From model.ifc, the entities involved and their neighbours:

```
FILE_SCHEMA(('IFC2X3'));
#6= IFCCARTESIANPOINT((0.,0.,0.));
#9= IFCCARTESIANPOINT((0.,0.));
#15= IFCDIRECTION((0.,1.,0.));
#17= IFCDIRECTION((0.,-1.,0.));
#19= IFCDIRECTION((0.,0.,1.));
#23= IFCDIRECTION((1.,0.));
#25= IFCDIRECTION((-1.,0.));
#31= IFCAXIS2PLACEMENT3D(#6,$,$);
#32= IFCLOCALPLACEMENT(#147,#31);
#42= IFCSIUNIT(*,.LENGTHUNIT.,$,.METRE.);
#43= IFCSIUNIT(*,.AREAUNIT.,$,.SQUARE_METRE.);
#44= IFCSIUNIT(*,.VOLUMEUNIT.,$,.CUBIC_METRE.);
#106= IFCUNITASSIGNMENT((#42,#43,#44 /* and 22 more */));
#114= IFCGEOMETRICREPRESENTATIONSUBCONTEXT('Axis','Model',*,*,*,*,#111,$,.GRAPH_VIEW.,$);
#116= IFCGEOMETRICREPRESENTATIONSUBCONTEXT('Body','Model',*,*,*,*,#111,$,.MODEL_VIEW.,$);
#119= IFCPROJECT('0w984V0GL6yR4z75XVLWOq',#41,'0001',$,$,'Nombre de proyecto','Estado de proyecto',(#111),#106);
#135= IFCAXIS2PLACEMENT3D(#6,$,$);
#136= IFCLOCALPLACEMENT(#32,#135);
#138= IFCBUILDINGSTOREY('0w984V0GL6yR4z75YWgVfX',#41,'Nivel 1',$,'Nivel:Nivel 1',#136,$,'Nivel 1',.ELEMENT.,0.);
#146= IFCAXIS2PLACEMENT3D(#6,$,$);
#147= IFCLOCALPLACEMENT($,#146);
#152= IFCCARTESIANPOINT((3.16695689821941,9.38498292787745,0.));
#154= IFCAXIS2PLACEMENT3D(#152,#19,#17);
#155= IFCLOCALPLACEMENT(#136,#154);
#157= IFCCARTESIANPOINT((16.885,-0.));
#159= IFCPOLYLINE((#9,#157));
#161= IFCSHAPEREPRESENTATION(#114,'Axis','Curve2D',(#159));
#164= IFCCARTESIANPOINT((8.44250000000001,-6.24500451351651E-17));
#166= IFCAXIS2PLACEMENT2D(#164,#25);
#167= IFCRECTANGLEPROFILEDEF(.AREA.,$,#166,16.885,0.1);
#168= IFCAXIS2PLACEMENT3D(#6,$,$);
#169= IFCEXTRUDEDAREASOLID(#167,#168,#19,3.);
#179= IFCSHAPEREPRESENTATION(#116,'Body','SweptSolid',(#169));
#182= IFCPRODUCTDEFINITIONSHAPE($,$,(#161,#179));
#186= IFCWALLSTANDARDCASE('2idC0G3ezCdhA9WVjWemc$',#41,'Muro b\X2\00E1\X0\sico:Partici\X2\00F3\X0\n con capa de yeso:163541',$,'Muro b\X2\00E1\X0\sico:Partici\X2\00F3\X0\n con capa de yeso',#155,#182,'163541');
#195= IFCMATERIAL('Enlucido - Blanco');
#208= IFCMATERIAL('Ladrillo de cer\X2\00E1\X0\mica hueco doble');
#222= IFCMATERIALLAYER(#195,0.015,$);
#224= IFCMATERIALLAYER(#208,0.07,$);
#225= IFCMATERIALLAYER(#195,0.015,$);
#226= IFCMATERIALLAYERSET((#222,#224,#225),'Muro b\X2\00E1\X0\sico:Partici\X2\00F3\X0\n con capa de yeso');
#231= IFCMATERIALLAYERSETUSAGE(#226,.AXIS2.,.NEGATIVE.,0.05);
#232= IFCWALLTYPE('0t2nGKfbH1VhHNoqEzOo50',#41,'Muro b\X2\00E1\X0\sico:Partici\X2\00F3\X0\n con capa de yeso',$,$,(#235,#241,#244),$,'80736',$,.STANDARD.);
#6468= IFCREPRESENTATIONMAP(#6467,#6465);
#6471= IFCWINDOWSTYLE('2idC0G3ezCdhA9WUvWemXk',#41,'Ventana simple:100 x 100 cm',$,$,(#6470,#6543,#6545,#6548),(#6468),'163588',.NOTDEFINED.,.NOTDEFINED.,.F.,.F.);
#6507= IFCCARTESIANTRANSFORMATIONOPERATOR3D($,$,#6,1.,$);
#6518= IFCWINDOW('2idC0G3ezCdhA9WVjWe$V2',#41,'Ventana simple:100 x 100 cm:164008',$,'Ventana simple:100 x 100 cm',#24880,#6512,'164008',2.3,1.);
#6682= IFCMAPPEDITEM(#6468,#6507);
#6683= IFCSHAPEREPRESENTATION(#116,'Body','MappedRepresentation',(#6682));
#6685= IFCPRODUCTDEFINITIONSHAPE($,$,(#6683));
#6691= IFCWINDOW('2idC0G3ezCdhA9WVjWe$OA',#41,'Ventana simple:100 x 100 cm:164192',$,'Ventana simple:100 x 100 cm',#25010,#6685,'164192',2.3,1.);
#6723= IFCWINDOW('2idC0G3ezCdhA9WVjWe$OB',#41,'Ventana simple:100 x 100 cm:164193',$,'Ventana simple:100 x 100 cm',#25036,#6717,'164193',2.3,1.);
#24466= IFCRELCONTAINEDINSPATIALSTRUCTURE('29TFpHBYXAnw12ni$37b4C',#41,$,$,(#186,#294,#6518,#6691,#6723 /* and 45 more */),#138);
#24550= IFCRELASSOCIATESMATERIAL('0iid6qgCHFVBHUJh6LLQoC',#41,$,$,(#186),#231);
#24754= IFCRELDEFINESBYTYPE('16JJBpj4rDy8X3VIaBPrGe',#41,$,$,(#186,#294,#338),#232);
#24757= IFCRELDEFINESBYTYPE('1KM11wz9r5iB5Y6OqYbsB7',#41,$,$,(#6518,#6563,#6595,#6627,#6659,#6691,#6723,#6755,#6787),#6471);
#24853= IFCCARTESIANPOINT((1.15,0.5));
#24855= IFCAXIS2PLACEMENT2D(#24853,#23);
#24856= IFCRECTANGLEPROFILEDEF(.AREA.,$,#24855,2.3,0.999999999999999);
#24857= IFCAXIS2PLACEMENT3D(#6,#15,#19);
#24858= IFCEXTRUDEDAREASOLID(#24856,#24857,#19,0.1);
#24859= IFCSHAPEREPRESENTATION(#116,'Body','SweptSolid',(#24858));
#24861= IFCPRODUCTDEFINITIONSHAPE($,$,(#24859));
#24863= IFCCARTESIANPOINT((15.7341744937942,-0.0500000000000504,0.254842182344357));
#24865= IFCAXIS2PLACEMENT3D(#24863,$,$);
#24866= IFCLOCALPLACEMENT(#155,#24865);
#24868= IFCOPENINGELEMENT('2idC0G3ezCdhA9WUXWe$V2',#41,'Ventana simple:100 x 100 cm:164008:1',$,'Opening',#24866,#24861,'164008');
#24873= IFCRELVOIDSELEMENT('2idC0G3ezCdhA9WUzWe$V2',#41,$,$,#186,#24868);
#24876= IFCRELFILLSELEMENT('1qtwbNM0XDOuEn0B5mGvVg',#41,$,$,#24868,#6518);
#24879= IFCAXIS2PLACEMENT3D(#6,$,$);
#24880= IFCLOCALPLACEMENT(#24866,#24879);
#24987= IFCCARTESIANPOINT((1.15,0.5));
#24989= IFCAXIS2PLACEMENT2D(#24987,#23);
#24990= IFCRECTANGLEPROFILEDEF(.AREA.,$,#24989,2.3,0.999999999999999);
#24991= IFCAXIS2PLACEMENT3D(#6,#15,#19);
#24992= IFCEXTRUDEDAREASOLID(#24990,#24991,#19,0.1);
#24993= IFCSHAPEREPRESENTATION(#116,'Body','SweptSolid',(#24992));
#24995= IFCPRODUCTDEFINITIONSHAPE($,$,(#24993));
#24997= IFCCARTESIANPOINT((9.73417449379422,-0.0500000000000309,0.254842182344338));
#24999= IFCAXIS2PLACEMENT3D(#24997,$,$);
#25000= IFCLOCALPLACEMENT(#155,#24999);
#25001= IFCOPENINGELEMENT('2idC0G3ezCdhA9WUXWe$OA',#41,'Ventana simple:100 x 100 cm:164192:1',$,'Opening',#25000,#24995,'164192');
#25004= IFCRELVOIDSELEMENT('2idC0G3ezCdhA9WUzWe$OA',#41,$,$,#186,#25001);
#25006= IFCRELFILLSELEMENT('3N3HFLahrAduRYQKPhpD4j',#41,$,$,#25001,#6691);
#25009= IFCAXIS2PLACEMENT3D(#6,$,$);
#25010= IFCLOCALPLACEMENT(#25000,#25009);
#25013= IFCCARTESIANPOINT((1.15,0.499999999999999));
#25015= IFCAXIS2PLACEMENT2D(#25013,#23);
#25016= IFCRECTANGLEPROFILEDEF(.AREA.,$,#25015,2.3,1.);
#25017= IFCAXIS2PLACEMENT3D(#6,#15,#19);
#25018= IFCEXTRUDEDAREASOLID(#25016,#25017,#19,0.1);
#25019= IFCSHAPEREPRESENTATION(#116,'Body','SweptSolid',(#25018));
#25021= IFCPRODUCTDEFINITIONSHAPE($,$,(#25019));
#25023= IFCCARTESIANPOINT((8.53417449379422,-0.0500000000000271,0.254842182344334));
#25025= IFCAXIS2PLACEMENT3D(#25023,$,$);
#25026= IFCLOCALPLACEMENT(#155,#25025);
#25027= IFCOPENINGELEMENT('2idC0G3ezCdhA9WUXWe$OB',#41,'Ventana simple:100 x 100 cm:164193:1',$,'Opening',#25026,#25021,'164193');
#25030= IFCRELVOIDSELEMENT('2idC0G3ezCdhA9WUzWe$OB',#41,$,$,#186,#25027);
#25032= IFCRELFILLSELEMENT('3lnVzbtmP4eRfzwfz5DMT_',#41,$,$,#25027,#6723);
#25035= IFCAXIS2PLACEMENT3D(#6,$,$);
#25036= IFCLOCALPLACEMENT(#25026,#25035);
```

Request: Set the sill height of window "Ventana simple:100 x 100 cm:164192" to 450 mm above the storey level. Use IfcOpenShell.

```python
import numpy as np
import ifcopenshell
import ifcopenshell.api.geometry
import ifcopenshell.geom
import ifcopenshell.util.element
import ifcopenshell.util.placement
import ifcopenshell.util.shape
import ifcopenshell.util.unit

model = ifcopenshell.open("model.ifc")
unit_scale = ifcopenshell.util.unit.calculate_unit_scale(model)

window = model.by_guid("2idC0G3ezCdhA9WVjWe$OA")
opening = window.FillsVoids[0].RelatingOpeningElement
storey = ifcopenshell.util.element.get_container(window, ifc_class="IfcBuildingStorey")
level = ifcopenshell.util.placement.get_local_placement(storey.ObjectPlacement)[2, 3]

# The opening's origin need not be at the sill, so measure its lowest point.
shape = ifcopenshell.geom.create_shape(ifcopenshell.geom.settings(), opening)
bottom = ifcopenshell.util.shape.get_shape_bottom_elevation(shape, shape.geometry) / unit_scale
dz = level + 0.45 - bottom

shift = np.array([0.0, 0.0, dz])
# The window is placed relative to its opening, so it follows when the opening moves.
matrix = ifcopenshell.util.placement.get_local_placement(opening.ObjectPlacement)
matrix[:3, 3] += shift
ifcopenshell.api.geometry.edit_object_placement(
    model, product=opening, matrix=matrix, is_si=False, should_transform_children=True
)

print(f"moved by {dz * unit_scale:+.3f} m")

model.write("model_rev.ifc")
```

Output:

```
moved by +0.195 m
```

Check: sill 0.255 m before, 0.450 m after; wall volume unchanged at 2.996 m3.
